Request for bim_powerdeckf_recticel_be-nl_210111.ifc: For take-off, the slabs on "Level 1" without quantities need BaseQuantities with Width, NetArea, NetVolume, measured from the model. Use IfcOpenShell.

First a look at what the model holds.

```python
import ifcopenshell
import ifcopenshell.util.element
import ifcopenshell.util.unit

model = ifcopenshell.open("bim_powerdeckf_recticel_be-nl_210111.ifc")
print(model.schema)
for unit_type in ("LENGTHUNIT", "AREAUNIT", "VOLUMEUNIT"):
    print(unit_type, ifcopenshell.util.unit.calculate_unit_scale(model, unit_type))
storey = next(s for s in model.by_type("IfcBuildingStorey") if s.Name == "Level 1")
slabs = [e for e in ifcopenshell.util.element.get_decomposition(storey) if e.is_a("IfcSlab")]
for e in sorted(slabs, key=lambda e: e.id()):
    print(e.id(), e.is_a(), e.Name, list(ifcopenshell.util.element.get_psets(e, qtos_only=True)), sep=" | ")
```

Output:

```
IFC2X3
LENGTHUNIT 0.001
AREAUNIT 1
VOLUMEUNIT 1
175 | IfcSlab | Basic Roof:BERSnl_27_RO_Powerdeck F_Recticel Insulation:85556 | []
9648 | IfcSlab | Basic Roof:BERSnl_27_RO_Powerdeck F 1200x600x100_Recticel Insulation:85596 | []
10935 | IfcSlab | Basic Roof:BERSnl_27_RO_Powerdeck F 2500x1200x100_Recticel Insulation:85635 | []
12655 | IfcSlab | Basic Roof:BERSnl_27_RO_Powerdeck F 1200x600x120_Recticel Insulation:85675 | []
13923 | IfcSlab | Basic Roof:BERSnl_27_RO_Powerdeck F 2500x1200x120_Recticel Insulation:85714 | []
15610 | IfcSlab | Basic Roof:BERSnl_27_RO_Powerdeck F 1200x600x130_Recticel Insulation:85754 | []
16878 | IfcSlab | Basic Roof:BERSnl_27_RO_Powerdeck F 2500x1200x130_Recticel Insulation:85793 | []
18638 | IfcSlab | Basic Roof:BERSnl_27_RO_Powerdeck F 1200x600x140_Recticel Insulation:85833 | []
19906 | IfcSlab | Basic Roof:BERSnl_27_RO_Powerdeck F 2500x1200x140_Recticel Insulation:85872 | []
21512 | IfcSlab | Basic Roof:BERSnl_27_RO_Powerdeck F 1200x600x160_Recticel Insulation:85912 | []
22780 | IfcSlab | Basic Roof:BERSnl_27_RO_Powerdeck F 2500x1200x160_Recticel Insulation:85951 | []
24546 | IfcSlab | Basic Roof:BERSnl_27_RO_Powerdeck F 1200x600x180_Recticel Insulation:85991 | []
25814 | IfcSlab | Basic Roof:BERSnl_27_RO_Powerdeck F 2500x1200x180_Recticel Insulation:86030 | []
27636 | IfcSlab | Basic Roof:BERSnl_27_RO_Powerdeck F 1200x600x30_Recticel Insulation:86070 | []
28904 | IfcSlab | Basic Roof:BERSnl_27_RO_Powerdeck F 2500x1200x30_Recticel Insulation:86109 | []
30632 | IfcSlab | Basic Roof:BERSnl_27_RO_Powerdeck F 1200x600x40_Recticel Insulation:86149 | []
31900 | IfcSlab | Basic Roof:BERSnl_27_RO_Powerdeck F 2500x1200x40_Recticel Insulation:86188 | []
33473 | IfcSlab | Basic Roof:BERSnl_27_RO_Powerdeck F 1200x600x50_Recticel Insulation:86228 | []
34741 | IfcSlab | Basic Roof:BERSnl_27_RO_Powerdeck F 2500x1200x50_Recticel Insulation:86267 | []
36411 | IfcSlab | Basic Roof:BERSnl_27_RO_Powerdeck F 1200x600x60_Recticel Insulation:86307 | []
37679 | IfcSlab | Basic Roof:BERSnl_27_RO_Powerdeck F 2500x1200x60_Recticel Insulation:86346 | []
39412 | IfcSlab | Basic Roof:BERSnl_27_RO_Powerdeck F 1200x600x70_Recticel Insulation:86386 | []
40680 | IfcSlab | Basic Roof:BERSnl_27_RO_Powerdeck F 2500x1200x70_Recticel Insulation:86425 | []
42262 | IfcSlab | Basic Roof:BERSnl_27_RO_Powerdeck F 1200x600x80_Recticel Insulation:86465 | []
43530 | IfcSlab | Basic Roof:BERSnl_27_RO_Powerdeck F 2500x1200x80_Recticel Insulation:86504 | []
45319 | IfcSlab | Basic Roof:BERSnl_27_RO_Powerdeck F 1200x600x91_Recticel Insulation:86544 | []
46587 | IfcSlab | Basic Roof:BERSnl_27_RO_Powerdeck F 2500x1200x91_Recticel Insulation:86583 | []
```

```python
import ifcopenshell
import ifcopenshell.api.pset
import ifcopenshell.geom
import ifcopenshell.util.element
import ifcopenshell.util.shape
import ifcopenshell.util.unit

model = ifcopenshell.open("bim_powerdeckf_recticel_be-nl_210111.ifc")
unit_scale = ifcopenshell.util.unit.calculate_unit_scale(model)
area_scale = ifcopenshell.util.unit.calculate_unit_scale(model, "AREAUNIT")
volume_scale = ifcopenshell.util.unit.calculate_unit_scale(model, "VOLUMEUNIT")
settings = ifcopenshell.geom.settings()

storey = next(s for s in model.by_type("IfcBuildingStorey") if s.Name == "Level 1")
slabs = [e for e in ifcopenshell.util.element.get_decomposition(storey) if e.is_a("IfcSlab")]

for e in sorted(slabs, key=lambda e: e.id()):
    if ifcopenshell.util.element.get_psets(e, qtos_only=True, should_inherit=False):
        continue
    # Geometry comes back in metres, in the element's own axes.
    shape = ifcopenshell.geom.create_shape(settings, e)
    values = {
        "Width": ifcopenshell.util.shape.get_z(shape.geometry) / unit_scale,
        "NetArea": ifcopenshell.util.shape.get_footprint_area(shape.geometry) / area_scale,
        "NetVolume": ifcopenshell.util.shape.get_volume(shape.geometry) / volume_scale,
    }
    qto = ifcopenshell.api.pset.add_qto(model, product=e, name="BaseQuantities")
    ifcopenshell.api.pset.edit_qto(model, qto=qto, properties=values)
    print(e.id(), {k: round(v, 3) for k, v in values.items()})

model.write("bim_powerdeckf_recticel_be-nl_210111_rev.ifc")
```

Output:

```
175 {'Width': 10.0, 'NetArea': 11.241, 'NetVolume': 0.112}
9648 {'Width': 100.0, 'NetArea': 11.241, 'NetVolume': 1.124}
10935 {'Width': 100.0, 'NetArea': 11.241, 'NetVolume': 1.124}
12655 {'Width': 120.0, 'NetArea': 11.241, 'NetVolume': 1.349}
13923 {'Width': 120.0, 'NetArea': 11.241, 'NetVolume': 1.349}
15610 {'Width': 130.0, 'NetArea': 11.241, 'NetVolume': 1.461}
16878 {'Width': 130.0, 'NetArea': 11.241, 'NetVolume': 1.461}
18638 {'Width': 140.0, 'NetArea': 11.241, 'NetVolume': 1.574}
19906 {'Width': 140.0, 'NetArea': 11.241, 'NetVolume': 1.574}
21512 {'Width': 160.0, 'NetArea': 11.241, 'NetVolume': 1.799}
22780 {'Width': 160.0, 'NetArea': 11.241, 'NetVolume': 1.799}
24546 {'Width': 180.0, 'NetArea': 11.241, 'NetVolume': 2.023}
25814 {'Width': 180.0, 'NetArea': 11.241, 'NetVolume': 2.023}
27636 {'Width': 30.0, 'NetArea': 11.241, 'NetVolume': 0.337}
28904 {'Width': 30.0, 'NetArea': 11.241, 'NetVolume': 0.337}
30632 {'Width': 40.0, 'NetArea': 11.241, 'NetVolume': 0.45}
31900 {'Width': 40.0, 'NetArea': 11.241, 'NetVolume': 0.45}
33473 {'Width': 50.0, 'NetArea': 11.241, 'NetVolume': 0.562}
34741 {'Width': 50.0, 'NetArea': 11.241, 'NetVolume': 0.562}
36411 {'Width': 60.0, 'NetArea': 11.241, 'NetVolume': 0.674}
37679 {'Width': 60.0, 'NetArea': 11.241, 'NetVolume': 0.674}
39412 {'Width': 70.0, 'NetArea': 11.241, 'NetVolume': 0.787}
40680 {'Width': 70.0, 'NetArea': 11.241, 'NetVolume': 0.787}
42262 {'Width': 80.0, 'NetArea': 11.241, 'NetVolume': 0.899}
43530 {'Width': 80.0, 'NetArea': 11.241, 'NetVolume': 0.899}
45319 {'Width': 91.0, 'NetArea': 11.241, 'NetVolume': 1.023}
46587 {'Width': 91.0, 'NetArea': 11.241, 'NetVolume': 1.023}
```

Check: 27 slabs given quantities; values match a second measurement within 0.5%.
